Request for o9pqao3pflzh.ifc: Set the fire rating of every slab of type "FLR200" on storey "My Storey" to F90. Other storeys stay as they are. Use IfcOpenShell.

First a look at what the model holds.

```python
import ifcopenshell
import ifcopenshell.util.element

model = ifcopenshell.open("o9pqao3pflzh.ifc")
print(model.schema)
storey = next(s for s in model.by_type("IfcBuildingStorey") if s.Name == "My Storey")
slabs = [e for e in ifcopenshell.util.element.get_decomposition(storey) if e.is_a("IfcSlab")]
seen = {}
for e in slabs:
    element_type = ifcopenshell.util.element.get_type(e)
    key = (element_type.Name if element_type != e and element_type else None, ifcopenshell.util.element.get_pset(e, "Pset_SlabCommon", "FireRating"))
    seen[key] = seen.get(key, 0) + 1
for (name, value), count in sorted(seen.items(), key=str):
    print(count, "x", name, "|", value)
```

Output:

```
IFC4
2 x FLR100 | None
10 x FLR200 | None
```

```python
import ifcopenshell
import ifcopenshell.api.pset
import ifcopenshell.util.element

model = ifcopenshell.open("o9pqao3pflzh.ifc")

storey = next(s for s in model.by_type("IfcBuildingStorey") if s.Name == "My Storey")
slabs = [e for e in ifcopenshell.util.element.get_decomposition(storey) if e.is_a("IfcSlab")]

count = 0
for e in slabs:
    element_type = ifcopenshell.util.element.get_type(e)
    if element_type in (None, e) or element_type.Name != "FLR200":
        continue
    # add_pset returns the element's existing set when there is one.
    pset = ifcopenshell.api.pset.add_pset(model, product=e, name="Pset_SlabCommon")
    ifcopenshell.api.pset.edit_pset(model, pset=pset, properties={"FireRating": "F90"})
    count += 1

print(count, "slabs updated")

model.write("o9pqao3pflzh-out.ifc")
```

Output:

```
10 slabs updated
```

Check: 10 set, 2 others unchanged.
